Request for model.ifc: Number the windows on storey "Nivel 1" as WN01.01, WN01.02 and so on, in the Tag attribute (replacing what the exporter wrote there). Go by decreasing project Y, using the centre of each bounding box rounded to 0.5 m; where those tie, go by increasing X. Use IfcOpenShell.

First a look at what the model holds.

```python
import ifcopenshell
import ifcopenshell.util.element
import ifcopenshell.util.placement

model = ifcopenshell.open("model.ifc")
print(model.schema)
storey = next(s for s in model.by_type("IfcBuildingStorey") if s.Name == "Nivel 1")
windows = [e for e in ifcopenshell.util.element.get_decomposition(storey) if e.is_a("IfcWindow")]
for e in sorted(windows, key=lambda e: e.id()):
    origin = ifcopenshell.util.placement.get_local_placement(e.ObjectPlacement)[:3, 3]
    print(e.id(), e.Tag, e.Name, origin.round(2) + 0.0, sep=" | ")
```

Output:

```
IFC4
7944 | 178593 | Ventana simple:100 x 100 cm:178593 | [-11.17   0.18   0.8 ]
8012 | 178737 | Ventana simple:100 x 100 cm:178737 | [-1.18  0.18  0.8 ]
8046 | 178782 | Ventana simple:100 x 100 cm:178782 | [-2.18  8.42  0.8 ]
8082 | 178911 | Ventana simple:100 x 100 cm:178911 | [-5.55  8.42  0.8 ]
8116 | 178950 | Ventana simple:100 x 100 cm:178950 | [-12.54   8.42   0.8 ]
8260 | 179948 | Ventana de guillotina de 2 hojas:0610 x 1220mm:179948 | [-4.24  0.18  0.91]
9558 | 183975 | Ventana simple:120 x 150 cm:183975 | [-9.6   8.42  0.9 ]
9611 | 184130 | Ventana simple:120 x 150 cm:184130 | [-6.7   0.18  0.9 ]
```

```python
import ifcopenshell
import ifcopenshell.geom
import ifcopenshell.util.element
import ifcopenshell.util.shape

model = ifcopenshell.open("model.ifc")
settings = ifcopenshell.geom.settings()
settings.set("use-world-coords", True)


def centre(element):
    shape = ifcopenshell.geom.create_shape(settings, element)
    return ifcopenshell.util.shape.get_bbox_centroid(shape.geometry)


storey = next(s for s in model.by_type("IfcBuildingStorey") if s.Name == "Nivel 1")
windows = [e for e in ifcopenshell.util.element.get_decomposition(storey) if e.is_a("IfcWindow")]

# Insertion points can sit at a corner or the storey origin, so sort by the geometry (in metres).
centres = {e: centre(e) for e in windows}
windows.sort(key=lambda e: (-round(centres[e][1] / 0.5), centres[e][0]))

for i, e in enumerate(windows, start=1):
    number = f"WN01.{i:02d}"
    e.Tag = number
    print(e.id(), number)

model.write("model_edited.ifc")
```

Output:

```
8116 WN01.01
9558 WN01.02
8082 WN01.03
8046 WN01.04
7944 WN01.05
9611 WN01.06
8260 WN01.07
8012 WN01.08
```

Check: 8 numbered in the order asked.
